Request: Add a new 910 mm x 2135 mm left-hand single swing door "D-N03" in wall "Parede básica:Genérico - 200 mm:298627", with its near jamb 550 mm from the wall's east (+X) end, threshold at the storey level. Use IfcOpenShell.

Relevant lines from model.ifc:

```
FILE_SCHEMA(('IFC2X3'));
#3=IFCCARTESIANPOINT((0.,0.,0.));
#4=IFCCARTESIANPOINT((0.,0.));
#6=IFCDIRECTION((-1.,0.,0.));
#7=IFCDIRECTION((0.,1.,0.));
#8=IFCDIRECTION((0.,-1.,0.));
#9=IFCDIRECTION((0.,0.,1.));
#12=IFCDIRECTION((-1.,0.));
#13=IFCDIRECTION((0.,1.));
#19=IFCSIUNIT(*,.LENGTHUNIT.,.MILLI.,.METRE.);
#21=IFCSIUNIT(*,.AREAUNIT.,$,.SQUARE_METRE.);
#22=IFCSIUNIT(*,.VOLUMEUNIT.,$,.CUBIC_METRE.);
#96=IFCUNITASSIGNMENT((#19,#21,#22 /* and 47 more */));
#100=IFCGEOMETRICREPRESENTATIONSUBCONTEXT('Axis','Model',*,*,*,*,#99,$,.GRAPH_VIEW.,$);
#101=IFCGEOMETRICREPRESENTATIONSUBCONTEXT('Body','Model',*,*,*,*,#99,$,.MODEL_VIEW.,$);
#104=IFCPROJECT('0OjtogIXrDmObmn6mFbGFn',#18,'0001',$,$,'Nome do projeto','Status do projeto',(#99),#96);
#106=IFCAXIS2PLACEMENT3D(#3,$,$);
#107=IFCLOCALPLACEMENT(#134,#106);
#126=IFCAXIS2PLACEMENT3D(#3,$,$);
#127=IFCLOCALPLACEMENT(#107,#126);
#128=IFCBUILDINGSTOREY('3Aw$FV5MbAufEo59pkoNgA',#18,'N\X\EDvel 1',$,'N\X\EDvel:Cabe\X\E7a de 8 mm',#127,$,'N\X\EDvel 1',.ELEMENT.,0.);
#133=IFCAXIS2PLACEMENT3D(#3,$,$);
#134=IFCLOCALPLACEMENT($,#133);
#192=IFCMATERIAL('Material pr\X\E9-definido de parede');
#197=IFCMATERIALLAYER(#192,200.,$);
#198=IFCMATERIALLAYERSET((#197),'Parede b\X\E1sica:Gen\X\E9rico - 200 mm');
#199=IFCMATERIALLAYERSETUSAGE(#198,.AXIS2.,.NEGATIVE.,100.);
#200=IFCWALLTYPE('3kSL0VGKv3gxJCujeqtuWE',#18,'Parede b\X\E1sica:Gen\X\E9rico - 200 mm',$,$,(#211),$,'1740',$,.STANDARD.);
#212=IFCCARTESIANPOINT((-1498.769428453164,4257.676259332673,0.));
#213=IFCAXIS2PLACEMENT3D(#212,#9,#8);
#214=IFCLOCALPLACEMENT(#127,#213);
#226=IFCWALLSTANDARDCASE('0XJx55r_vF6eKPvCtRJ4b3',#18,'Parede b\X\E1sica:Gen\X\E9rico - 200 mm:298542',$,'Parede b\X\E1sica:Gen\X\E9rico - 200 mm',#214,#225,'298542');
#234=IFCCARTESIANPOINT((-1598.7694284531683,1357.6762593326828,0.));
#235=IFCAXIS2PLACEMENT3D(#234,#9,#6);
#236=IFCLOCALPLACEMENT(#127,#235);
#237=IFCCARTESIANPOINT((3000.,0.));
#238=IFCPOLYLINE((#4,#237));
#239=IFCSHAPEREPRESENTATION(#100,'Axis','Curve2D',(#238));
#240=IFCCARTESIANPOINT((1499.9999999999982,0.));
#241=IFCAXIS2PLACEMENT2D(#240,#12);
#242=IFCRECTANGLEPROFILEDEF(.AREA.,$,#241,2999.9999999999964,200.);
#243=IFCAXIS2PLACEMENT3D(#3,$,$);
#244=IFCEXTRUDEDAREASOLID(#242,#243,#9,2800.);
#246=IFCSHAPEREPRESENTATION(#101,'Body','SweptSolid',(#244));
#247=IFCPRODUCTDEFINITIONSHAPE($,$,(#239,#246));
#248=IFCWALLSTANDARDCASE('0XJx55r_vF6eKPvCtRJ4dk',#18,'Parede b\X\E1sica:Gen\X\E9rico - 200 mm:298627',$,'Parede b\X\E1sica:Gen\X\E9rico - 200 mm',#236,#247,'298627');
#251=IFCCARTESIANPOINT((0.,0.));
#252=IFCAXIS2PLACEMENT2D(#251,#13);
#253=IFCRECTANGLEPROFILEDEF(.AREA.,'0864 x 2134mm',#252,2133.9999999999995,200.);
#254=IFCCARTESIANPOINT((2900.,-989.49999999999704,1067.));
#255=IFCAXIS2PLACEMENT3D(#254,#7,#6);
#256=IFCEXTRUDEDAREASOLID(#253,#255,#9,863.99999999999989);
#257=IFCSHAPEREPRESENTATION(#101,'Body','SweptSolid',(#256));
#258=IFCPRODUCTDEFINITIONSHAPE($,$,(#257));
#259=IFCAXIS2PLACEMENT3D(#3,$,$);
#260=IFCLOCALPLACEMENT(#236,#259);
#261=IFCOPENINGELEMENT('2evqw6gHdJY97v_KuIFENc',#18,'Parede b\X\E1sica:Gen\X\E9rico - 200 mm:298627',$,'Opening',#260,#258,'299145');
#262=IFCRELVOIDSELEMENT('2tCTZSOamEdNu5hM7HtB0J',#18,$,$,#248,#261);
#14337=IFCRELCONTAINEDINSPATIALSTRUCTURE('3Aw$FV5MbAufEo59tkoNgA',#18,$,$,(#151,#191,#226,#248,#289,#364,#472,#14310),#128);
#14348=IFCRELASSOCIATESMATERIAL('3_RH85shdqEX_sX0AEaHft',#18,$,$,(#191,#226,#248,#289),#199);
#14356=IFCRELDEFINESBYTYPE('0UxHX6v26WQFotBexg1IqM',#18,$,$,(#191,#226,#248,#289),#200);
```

```python
import numpy as np
import ifcopenshell
import ifcopenshell.api.feature
import ifcopenshell.api.geometry
import ifcopenshell.api.root
import ifcopenshell.api.spatial
import ifcopenshell.api.type
import ifcopenshell.geom
import ifcopenshell.util.element
import ifcopenshell.util.placement
import ifcopenshell.util.representation
import ifcopenshell.util.shape
import ifcopenshell.util.unit

model = ifcopenshell.open("model.ifc")
unit_scale = ifcopenshell.util.unit.calculate_unit_scale(model)
settings = ifcopenshell.geom.settings()


def volume(element):
    """Net volume in cubic metres, openings subtracted."""
    shape = ifcopenshell.geom.create_shape(settings, element)
    return ifcopenshell.util.shape.get_volume(shape.geometry)


wall = model.by_guid("0XJx55r_vF6eKPvCtRJ4dk")
storey = ifcopenshell.util.element.get_container(wall, ifc_class="IfcBuildingStorey")
context = ifcopenshell.util.representation.get_context(model, "Model", "Body", "MODEL_VIEW")
before = volume(wall)

width, height, from_end, sill = 0.91, 2.135, 0.55, 0.0  # metres

# The wall runs along its own X axis, and the end named is its -X end.
wall_shape = ifcopenshell.geom.create_shape(settings, wall)
x, y, z = ifcopenshell.util.shape.get_vertices(wall_shape.geometry).T
start = x.min() + from_end
face, thickness = float(y.min()), float(y.max() - y.min())
wall_matrix = ifcopenshell.util.placement.get_local_placement(wall.ObjectPlacement)
level = ifcopenshell.util.placement.get_local_placement(storey.ObjectPlacement)[2, 3]


def in_wall(x, y):
    """Placement at x, y metres in the wall's axes, at sill height."""
    matrix = wall_matrix.copy()
    matrix[:, 3] = wall_matrix @ np.array([x / unit_scale, y / unit_scale, 0.0, 1.0])
    matrix[2, 3] = level + sill / unit_scale
    return matrix


# Opening: a box that overshoots both wall faces by 50 mm.
opening = ifcopenshell.api.root.create_entity(model, ifc_class="IfcOpeningElement")
box = ifcopenshell.api.geometry.add_wall_representation(
    model, context=context, length=width, height=height, thickness=thickness + 0.1
)
ifcopenshell.api.geometry.assign_representation(model, product=opening, representation=box)
ifcopenshell.api.geometry.edit_object_placement(model, product=opening, matrix=in_wall(start, face - 0.05), is_si=False)
ifcopenshell.api.feature.add_feature(model, feature=opening, element=wall)

door = ifcopenshell.api.root.create_entity(model, ifc_class="IfcDoor", name="D-N03")
door.OverallWidth, door.OverallHeight = width / unit_scale, height / unit_scale
body = ifcopenshell.api.geometry.add_door_representation(
    model,
    context=context,
    overall_width=door.OverallWidth,
    overall_height=door.OverallHeight,
    operation_type="SINGLE_SWING_LEFT",
    lining_properties={"LiningDepth": thickness / unit_scale, "ThresholdDepth": thickness / unit_scale},
)
ifcopenshell.api.geometry.assign_representation(model, product=door, representation=body)
ifcopenshell.api.spatial.assign_container(model, products=[door], relating_structure=storey)
fills = ifcopenshell.api.feature.add_filling(model, opening=opening, element=door)
fills.OwnerHistory = door.OwnerHistory  # required in IFC2X3

# IFC2X3 keeps the operation on the door style.
style = ifcopenshell.api.root.create_entity(model, ifc_class="IfcDoorStyle", name="D-N03")
style.OperationType, style.ConstructionType = "SINGLE_SWING_LEFT", "NOTDEFINED"
style.ParameterTakesPrecedence = style.Sizeable = False
ifcopenshell.api.type.assign_type(model, related_objects=[door], relating_type=style)

# The lining spans the wall, so the door starts at the wall face.
ifcopenshell.api.geometry.edit_object_placement(model, product=door, matrix=in_wall(start, face), is_si=False)

after = volume(wall)

print(f"wall volume {before:.3f} -> {after:.3f} m3")

model.write("model-out.ifc")
```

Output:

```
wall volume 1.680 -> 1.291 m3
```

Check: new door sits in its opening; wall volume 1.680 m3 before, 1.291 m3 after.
